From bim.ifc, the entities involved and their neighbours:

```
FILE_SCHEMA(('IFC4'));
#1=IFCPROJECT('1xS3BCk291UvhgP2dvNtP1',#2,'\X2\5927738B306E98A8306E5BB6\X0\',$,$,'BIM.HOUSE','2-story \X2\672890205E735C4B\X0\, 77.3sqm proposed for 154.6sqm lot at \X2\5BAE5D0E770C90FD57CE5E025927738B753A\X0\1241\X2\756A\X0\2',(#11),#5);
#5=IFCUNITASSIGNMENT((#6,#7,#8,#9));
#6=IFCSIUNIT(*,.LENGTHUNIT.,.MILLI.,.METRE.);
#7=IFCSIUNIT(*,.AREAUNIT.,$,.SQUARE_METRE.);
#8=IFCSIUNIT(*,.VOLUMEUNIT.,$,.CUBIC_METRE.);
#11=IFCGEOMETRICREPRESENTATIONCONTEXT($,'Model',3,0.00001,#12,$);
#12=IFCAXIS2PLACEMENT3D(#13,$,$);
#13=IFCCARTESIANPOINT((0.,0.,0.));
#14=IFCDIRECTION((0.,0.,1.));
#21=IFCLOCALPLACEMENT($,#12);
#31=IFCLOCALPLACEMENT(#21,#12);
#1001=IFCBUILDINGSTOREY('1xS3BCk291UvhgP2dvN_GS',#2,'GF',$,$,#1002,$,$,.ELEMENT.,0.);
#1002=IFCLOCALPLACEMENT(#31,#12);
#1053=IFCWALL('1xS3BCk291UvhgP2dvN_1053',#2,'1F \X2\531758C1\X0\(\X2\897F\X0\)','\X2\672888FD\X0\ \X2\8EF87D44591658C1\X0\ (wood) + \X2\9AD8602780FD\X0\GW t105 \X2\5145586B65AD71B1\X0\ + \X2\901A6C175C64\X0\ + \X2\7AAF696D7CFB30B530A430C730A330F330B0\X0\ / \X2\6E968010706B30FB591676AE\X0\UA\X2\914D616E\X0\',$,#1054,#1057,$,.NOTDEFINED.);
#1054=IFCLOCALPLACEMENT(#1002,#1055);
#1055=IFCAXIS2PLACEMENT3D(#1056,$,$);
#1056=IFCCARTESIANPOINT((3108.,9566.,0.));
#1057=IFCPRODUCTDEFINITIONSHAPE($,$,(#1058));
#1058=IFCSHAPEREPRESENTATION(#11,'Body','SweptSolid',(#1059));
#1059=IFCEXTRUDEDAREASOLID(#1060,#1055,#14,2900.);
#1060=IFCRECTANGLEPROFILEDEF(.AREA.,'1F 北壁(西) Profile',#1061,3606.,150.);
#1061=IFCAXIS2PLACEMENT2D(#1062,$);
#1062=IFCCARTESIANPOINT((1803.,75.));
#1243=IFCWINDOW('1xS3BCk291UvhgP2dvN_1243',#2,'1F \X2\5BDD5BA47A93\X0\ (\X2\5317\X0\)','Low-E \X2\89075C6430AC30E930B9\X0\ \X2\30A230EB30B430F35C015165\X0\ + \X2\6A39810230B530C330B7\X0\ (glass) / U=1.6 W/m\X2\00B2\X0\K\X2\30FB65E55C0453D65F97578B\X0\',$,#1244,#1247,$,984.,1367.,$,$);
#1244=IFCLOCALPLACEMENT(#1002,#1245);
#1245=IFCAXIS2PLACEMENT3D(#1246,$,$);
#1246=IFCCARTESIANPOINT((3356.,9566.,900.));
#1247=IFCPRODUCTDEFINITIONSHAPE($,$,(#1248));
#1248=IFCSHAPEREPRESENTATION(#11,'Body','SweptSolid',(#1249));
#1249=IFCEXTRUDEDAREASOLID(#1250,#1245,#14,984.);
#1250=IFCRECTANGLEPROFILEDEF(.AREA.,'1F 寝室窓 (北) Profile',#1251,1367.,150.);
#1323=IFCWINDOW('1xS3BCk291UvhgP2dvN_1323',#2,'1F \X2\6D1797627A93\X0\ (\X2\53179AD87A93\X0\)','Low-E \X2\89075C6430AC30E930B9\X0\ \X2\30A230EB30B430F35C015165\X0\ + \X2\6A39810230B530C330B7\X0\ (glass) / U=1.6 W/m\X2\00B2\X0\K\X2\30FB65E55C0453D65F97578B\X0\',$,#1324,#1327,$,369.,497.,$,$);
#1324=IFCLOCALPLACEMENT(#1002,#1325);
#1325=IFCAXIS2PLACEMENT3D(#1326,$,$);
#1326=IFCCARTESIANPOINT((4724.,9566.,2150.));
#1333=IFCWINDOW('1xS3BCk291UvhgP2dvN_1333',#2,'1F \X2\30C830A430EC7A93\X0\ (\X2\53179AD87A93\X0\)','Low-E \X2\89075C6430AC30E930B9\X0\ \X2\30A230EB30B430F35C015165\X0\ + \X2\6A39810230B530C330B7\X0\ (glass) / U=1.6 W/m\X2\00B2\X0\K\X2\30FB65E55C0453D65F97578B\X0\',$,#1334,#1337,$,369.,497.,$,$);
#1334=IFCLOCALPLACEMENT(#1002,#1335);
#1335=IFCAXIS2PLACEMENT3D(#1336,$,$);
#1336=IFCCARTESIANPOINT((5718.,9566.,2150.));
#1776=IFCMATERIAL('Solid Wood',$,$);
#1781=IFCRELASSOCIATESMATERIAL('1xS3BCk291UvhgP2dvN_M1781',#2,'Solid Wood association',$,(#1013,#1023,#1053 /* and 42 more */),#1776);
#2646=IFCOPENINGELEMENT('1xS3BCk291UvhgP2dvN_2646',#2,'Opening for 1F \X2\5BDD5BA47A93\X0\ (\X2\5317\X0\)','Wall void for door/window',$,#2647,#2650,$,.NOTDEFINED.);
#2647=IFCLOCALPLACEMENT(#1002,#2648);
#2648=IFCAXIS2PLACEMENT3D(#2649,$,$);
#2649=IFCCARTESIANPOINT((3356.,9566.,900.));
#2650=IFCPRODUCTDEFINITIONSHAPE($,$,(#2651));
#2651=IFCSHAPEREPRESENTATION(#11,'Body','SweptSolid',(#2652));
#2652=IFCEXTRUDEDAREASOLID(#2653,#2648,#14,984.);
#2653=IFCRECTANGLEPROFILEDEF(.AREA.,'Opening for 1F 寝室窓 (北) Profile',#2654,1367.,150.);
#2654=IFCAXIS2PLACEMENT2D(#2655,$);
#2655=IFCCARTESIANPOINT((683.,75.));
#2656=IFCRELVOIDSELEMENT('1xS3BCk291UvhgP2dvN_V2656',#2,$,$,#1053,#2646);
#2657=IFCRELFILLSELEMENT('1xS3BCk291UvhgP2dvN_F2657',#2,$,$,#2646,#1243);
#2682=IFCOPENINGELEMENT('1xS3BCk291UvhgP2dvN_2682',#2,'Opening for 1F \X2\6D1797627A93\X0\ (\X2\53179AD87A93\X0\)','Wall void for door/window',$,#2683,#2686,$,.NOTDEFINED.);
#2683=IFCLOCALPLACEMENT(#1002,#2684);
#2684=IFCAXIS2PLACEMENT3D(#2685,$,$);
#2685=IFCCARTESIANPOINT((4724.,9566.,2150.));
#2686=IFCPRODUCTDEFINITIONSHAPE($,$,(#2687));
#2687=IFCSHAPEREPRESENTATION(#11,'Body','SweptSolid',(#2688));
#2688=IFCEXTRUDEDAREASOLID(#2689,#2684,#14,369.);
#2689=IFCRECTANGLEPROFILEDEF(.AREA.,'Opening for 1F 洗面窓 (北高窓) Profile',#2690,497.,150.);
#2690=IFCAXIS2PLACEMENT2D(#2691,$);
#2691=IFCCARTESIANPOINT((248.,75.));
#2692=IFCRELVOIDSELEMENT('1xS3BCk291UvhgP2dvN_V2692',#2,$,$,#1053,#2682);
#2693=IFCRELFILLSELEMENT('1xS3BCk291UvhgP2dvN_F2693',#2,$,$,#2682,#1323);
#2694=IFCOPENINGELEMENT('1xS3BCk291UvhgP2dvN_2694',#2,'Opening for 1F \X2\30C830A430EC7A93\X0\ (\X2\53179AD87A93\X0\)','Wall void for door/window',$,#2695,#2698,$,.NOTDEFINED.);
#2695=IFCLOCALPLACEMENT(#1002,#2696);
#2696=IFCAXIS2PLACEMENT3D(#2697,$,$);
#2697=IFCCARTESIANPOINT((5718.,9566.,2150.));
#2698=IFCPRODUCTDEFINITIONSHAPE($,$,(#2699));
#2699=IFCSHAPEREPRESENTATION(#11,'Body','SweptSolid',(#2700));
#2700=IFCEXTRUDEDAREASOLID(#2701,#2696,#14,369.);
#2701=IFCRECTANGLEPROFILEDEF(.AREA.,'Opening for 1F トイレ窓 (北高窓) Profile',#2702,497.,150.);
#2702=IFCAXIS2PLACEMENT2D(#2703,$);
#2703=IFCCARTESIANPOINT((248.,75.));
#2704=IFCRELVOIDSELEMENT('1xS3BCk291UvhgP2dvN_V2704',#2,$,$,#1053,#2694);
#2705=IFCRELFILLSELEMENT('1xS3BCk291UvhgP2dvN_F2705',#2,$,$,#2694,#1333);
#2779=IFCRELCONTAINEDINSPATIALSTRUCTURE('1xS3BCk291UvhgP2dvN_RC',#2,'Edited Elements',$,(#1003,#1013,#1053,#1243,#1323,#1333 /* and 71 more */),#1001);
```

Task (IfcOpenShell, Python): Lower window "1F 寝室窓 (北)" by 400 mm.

```python
import numpy as np
import ifcopenshell
import ifcopenshell.api.geometry
import ifcopenshell.util.placement
import ifcopenshell.util.unit

model = ifcopenshell.open("bim.ifc")
unit_scale = ifcopenshell.util.unit.calculate_unit_scale(model)

window = model.by_guid("1xS3BCk291UvhgP2dvN_1243")
opening = window.FillsVoids[0].RelatingOpeningElement
dz = -0.4 / unit_scale

shift = np.array([0.0, 0.0, dz])
# The window is not placed relative to its opening, so move both.
for product in (opening, window):
    matrix = ifcopenshell.util.placement.get_local_placement(product.ObjectPlacement)
    matrix[:3, 3] += shift
    ifcopenshell.api.geometry.edit_object_placement(model, product=product, matrix=matrix, is_si=False)

print(f"moved by {dz * unit_scale:+.3f} m")

model.write("bim_rev.ifc")
```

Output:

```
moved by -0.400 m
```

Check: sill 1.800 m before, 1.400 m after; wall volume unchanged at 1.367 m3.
